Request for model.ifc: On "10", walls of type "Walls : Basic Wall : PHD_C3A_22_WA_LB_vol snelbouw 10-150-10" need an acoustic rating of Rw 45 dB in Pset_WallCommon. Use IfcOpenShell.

First a look at what the model holds.

```python
import ifcopenshell
import ifcopenshell.util.element

model = ifcopenshell.open("model.ifc")
print(model.schema)
storey = next(s for s in model.by_type("IfcBuildingStorey") if s.Name == "10")
walls = [e for e in ifcopenshell.util.element.get_decomposition(storey) if e.is_a("IfcWall")]
seen = {}
for e in walls:
    element_type = ifcopenshell.util.element.get_type(e)
    key = (element_type.Name if element_type != e and element_type else None, ifcopenshell.util.element.get_pset(e, "Pset_WallCommon", "AcousticRating"))
    seen[key] = seen.get(key, 0) + 1
for (name, value), count in sorted(seen.items(), key=str):
    print(count, "x", name, "|", value)
```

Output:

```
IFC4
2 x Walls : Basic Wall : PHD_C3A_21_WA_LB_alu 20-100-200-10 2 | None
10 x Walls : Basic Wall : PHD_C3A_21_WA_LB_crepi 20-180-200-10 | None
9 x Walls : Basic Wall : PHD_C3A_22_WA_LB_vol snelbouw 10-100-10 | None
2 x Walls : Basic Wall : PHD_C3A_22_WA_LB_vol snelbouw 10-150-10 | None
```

```python
import ifcopenshell
import ifcopenshell.api.pset
import ifcopenshell.util.element

model = ifcopenshell.open("model.ifc")

storey = next(s for s in model.by_type("IfcBuildingStorey") if s.Name == "10")
walls = [e for e in ifcopenshell.util.element.get_decomposition(storey) if e.is_a("IfcWall")]

count = 0
for e in walls:
    element_type = ifcopenshell.util.element.get_type(e)
    if element_type in (None, e) or element_type.Name != "Walls : Basic Wall : PHD_C3A_22_WA_LB_vol snelbouw 10-150-10":
        continue
    # add_pset returns the element's existing set when there is one.
    pset = ifcopenshell.api.pset.add_pset(model, product=e, name="Pset_WallCommon")
    ifcopenshell.api.pset.edit_pset(model, pset=pset, properties={"AcousticRating": "Rw 45 dB"})
    count += 1

print(count, "walls updated")

model.write("model_edited.ifc")
```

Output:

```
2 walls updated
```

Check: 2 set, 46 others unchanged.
